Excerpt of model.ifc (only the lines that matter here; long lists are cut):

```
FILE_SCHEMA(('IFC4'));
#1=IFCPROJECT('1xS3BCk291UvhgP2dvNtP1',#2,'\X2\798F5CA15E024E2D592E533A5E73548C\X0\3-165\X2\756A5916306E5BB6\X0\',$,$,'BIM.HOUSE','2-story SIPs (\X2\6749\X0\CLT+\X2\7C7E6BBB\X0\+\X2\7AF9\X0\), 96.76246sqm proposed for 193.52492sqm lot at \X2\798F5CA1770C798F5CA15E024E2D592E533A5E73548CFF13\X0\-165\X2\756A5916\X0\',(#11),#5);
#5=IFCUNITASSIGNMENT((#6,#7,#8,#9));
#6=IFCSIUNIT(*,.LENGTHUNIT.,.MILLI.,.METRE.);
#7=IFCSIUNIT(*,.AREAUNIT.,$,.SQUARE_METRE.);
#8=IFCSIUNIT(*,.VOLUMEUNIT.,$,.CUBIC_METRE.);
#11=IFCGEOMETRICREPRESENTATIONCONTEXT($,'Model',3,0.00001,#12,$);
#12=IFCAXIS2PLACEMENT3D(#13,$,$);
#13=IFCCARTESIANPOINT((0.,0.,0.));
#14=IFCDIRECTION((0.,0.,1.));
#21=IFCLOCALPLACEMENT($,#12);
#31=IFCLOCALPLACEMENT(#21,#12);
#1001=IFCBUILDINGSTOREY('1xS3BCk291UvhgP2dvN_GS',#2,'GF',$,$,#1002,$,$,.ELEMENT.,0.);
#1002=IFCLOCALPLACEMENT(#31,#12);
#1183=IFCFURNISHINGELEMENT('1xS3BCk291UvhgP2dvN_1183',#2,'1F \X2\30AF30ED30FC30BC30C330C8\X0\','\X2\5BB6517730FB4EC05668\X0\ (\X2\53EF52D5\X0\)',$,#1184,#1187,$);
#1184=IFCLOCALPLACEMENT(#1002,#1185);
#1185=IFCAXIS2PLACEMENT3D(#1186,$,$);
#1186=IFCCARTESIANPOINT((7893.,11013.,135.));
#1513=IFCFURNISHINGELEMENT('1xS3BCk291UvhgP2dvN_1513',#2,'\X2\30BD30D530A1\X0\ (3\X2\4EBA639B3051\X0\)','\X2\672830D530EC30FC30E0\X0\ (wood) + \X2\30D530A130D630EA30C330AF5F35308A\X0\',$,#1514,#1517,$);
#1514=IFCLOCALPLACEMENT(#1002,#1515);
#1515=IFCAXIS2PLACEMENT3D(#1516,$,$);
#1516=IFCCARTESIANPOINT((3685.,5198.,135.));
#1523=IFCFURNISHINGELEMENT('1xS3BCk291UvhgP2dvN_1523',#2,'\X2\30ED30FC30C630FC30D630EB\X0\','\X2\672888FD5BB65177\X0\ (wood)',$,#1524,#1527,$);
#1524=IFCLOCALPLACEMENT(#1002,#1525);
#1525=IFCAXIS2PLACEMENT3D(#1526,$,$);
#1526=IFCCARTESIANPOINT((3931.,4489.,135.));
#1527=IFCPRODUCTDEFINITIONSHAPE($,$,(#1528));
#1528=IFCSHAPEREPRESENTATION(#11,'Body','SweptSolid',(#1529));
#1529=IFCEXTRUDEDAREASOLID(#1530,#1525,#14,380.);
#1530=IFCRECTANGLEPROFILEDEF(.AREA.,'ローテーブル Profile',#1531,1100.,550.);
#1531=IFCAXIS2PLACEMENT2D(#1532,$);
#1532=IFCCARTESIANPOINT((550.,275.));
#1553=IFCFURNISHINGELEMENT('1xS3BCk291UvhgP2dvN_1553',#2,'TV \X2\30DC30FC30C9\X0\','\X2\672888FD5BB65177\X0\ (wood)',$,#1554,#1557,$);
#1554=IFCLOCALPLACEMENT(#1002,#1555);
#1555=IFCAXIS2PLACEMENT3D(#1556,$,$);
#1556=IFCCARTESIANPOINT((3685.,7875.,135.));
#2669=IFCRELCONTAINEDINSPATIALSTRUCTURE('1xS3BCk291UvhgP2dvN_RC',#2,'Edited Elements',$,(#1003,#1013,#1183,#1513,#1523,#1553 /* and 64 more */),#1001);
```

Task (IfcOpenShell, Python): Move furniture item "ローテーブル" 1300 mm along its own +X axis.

```python
import ifcopenshell
import ifcopenshell.api.geometry
import ifcopenshell.util.placement
import ifcopenshell.util.unit

model = ifcopenshell.open("model.ifc")
unit_scale = ifcopenshell.util.unit.calculate_unit_scale(model)

item = model.by_guid("1xS3BCk291UvhgP2dvN_1523")
matrix = ifcopenshell.util.placement.get_local_placement(item.ObjectPlacement)
matrix[:3, 3] += matrix[:3, 0] * 1.3 / unit_scale
ifcopenshell.api.geometry.edit_object_placement(model, product=item, matrix=matrix, is_si=False)

print(ifcopenshell.util.placement.get_local_placement(item.ObjectPlacement).round(3) + 0.0)

model.write("model_v2.ifc")
```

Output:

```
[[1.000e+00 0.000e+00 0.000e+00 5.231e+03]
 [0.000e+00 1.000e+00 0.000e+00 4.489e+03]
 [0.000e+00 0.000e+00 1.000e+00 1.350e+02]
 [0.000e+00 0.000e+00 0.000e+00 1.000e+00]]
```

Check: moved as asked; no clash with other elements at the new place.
